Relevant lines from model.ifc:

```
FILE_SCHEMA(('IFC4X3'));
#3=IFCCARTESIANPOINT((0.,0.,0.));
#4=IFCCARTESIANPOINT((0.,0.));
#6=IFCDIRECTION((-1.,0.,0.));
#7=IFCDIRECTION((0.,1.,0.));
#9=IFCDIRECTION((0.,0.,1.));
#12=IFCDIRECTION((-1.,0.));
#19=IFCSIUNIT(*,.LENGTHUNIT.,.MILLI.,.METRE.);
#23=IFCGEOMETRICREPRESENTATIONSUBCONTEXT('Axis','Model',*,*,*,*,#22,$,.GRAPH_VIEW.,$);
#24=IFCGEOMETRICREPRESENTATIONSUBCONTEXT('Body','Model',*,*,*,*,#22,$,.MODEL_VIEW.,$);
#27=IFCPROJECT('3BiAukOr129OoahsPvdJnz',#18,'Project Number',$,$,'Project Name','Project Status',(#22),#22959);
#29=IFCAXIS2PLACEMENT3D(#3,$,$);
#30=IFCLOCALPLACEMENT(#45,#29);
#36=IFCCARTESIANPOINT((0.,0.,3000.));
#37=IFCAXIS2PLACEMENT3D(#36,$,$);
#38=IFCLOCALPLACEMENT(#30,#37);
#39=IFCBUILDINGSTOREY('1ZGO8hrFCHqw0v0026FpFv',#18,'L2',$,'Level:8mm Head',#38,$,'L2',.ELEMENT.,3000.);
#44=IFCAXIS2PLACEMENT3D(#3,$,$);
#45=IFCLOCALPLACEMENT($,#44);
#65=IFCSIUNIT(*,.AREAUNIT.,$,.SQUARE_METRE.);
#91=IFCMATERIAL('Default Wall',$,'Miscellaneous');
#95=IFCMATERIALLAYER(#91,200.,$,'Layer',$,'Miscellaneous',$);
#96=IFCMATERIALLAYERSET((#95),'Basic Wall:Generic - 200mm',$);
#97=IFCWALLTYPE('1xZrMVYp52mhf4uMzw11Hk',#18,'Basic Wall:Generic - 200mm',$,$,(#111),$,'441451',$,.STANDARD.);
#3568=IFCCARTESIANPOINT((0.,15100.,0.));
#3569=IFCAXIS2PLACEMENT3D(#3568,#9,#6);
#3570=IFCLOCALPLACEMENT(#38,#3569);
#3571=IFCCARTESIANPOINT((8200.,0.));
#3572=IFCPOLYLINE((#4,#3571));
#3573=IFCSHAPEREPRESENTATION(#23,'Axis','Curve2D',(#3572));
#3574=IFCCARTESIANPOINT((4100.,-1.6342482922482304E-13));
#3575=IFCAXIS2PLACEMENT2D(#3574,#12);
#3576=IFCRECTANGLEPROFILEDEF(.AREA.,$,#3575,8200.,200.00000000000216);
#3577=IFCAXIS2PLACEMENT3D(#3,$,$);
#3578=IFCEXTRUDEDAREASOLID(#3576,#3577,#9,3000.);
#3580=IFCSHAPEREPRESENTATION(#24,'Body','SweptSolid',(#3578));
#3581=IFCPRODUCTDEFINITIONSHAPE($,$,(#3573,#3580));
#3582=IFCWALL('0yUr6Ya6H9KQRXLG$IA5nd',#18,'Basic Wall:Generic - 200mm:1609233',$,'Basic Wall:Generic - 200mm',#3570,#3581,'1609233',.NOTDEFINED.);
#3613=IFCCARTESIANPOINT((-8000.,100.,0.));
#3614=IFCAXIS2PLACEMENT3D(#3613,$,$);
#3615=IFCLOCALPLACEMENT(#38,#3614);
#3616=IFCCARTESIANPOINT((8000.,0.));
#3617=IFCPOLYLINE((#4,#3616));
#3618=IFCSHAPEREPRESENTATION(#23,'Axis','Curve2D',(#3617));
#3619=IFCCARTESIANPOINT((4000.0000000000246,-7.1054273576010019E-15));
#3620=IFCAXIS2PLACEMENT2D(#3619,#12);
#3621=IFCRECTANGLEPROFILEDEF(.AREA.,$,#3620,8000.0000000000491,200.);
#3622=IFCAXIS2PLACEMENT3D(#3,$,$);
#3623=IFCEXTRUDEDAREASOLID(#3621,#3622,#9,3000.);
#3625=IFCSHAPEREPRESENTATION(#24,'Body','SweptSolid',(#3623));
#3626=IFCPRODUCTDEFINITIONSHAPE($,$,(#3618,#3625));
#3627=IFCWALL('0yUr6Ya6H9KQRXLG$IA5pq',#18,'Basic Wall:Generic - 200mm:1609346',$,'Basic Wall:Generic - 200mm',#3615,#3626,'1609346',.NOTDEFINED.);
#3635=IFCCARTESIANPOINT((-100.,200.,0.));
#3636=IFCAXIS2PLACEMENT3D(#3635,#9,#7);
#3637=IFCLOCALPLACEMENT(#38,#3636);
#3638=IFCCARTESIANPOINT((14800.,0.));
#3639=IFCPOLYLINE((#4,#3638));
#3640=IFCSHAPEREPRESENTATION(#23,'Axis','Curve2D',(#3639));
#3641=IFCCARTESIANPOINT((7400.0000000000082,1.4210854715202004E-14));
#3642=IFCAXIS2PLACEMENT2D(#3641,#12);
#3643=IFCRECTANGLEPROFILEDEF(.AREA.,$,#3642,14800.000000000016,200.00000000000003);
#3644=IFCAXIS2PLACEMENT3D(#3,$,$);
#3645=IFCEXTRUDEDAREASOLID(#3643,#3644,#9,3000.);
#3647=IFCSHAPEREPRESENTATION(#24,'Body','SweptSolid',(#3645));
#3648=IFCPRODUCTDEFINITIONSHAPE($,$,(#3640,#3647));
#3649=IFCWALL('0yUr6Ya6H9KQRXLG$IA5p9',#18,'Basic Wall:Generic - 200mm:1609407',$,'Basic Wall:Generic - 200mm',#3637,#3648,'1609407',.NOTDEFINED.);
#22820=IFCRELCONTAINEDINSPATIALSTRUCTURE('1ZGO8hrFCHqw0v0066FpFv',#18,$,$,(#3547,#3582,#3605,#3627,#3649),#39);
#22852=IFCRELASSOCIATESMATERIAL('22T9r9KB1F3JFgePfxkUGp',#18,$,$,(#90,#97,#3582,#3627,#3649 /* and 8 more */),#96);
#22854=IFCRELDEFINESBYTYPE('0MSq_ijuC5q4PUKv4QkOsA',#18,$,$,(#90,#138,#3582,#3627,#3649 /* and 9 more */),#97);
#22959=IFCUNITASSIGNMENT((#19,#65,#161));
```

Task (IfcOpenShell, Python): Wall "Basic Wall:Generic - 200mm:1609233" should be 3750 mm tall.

```python
import ifcopenshell
import ifcopenshell.geom
import ifcopenshell.util.representation
import ifcopenshell.util.shape
import ifcopenshell.util.unit

model = ifcopenshell.open("model.ifc")
unit_scale = ifcopenshell.util.unit.calculate_unit_scale(model)
settings = ifcopenshell.geom.settings()


def volume(element):
    """Net volume in cubic metres, openings subtracted."""
    shape = ifcopenshell.geom.create_shape(settings, element)
    return ifcopenshell.util.shape.get_volume(shape.geometry)


wall = model.by_guid("0yUr6Ya6H9KQRXLG$IA5nd")
before = volume(wall)

body = ifcopenshell.util.representation.get_representation(wall, "Model", "Body")
solid = body.Items[0]
old_height = solid.Depth
solid.Depth = 3.75 / unit_scale
after = volume(wall)

print(f"height {old_height:g} -> {solid.Depth:g}, volume {before:.3f} -> {after:.3f} m3")

model.write("model_edited.ifc")
```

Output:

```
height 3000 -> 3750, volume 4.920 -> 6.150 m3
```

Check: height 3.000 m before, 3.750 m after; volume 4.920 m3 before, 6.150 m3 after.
